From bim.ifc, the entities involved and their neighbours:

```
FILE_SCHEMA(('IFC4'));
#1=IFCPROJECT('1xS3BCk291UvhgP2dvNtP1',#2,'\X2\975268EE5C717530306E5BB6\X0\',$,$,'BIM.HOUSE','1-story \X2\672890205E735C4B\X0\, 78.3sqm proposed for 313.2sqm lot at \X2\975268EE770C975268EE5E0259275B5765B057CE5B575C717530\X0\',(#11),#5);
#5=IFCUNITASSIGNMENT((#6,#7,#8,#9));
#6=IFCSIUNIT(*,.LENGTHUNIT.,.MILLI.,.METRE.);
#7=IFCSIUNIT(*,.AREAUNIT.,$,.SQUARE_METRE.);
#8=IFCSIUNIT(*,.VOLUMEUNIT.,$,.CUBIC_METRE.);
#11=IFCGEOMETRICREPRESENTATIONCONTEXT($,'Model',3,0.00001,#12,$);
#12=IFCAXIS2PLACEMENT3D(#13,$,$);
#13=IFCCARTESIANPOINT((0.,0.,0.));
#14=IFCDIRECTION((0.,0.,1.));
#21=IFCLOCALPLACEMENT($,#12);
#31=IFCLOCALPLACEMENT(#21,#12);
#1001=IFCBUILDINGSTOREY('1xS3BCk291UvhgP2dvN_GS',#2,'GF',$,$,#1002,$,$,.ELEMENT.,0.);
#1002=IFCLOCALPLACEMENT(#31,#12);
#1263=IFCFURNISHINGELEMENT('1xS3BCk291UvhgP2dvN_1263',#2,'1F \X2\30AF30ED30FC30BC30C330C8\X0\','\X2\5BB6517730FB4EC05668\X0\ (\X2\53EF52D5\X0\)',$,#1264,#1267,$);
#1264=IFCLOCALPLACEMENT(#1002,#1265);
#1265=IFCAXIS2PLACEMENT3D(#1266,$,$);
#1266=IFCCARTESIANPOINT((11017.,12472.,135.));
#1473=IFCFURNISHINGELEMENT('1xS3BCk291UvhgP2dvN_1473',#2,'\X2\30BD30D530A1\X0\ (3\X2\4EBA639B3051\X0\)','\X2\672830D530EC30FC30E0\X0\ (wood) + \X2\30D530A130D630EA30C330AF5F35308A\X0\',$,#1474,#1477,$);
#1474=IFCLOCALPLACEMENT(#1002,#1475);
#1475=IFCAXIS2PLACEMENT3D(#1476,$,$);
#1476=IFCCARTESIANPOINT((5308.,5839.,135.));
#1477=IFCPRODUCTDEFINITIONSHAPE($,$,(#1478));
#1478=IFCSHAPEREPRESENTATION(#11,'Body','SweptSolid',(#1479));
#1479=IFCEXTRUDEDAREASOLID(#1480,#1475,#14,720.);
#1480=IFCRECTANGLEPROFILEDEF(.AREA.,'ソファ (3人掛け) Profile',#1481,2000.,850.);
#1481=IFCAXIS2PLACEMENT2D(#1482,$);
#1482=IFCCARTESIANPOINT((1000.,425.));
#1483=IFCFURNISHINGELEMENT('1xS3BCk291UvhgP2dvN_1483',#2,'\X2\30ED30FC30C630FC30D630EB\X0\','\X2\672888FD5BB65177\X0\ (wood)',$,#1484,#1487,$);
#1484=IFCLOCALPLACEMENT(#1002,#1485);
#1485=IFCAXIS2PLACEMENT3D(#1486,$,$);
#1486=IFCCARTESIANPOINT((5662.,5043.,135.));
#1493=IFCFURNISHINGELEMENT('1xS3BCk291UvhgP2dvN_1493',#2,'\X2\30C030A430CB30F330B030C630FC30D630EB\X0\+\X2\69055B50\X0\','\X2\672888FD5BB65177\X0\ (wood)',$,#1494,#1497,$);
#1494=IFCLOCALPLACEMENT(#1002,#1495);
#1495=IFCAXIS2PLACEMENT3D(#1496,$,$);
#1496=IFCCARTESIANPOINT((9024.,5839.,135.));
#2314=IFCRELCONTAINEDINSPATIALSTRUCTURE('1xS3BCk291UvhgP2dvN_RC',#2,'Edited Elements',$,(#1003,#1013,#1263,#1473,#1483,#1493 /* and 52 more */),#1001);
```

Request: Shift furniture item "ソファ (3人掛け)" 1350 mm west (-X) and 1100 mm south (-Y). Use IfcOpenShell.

```python
import ifcopenshell
import ifcopenshell.api.geometry
import ifcopenshell.util.placement

model = ifcopenshell.open("bim.ifc")

item = model.by_guid("1xS3BCk291UvhgP2dvN_1473")
matrix = ifcopenshell.util.placement.get_local_placement(item.ObjectPlacement)
matrix[0, 3] -= 1350.0
matrix[1, 3] -= 1100.0
ifcopenshell.api.geometry.edit_object_placement(model, product=item, matrix=matrix, is_si=False)

print(ifcopenshell.util.placement.get_local_placement(item.ObjectPlacement).round(3) + 0.0)

model.write("bim_v2.ifc")
```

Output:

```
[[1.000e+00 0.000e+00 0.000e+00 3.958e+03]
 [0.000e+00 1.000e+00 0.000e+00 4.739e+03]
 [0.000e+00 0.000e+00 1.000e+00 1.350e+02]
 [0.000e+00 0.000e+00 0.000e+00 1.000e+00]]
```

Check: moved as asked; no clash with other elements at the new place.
